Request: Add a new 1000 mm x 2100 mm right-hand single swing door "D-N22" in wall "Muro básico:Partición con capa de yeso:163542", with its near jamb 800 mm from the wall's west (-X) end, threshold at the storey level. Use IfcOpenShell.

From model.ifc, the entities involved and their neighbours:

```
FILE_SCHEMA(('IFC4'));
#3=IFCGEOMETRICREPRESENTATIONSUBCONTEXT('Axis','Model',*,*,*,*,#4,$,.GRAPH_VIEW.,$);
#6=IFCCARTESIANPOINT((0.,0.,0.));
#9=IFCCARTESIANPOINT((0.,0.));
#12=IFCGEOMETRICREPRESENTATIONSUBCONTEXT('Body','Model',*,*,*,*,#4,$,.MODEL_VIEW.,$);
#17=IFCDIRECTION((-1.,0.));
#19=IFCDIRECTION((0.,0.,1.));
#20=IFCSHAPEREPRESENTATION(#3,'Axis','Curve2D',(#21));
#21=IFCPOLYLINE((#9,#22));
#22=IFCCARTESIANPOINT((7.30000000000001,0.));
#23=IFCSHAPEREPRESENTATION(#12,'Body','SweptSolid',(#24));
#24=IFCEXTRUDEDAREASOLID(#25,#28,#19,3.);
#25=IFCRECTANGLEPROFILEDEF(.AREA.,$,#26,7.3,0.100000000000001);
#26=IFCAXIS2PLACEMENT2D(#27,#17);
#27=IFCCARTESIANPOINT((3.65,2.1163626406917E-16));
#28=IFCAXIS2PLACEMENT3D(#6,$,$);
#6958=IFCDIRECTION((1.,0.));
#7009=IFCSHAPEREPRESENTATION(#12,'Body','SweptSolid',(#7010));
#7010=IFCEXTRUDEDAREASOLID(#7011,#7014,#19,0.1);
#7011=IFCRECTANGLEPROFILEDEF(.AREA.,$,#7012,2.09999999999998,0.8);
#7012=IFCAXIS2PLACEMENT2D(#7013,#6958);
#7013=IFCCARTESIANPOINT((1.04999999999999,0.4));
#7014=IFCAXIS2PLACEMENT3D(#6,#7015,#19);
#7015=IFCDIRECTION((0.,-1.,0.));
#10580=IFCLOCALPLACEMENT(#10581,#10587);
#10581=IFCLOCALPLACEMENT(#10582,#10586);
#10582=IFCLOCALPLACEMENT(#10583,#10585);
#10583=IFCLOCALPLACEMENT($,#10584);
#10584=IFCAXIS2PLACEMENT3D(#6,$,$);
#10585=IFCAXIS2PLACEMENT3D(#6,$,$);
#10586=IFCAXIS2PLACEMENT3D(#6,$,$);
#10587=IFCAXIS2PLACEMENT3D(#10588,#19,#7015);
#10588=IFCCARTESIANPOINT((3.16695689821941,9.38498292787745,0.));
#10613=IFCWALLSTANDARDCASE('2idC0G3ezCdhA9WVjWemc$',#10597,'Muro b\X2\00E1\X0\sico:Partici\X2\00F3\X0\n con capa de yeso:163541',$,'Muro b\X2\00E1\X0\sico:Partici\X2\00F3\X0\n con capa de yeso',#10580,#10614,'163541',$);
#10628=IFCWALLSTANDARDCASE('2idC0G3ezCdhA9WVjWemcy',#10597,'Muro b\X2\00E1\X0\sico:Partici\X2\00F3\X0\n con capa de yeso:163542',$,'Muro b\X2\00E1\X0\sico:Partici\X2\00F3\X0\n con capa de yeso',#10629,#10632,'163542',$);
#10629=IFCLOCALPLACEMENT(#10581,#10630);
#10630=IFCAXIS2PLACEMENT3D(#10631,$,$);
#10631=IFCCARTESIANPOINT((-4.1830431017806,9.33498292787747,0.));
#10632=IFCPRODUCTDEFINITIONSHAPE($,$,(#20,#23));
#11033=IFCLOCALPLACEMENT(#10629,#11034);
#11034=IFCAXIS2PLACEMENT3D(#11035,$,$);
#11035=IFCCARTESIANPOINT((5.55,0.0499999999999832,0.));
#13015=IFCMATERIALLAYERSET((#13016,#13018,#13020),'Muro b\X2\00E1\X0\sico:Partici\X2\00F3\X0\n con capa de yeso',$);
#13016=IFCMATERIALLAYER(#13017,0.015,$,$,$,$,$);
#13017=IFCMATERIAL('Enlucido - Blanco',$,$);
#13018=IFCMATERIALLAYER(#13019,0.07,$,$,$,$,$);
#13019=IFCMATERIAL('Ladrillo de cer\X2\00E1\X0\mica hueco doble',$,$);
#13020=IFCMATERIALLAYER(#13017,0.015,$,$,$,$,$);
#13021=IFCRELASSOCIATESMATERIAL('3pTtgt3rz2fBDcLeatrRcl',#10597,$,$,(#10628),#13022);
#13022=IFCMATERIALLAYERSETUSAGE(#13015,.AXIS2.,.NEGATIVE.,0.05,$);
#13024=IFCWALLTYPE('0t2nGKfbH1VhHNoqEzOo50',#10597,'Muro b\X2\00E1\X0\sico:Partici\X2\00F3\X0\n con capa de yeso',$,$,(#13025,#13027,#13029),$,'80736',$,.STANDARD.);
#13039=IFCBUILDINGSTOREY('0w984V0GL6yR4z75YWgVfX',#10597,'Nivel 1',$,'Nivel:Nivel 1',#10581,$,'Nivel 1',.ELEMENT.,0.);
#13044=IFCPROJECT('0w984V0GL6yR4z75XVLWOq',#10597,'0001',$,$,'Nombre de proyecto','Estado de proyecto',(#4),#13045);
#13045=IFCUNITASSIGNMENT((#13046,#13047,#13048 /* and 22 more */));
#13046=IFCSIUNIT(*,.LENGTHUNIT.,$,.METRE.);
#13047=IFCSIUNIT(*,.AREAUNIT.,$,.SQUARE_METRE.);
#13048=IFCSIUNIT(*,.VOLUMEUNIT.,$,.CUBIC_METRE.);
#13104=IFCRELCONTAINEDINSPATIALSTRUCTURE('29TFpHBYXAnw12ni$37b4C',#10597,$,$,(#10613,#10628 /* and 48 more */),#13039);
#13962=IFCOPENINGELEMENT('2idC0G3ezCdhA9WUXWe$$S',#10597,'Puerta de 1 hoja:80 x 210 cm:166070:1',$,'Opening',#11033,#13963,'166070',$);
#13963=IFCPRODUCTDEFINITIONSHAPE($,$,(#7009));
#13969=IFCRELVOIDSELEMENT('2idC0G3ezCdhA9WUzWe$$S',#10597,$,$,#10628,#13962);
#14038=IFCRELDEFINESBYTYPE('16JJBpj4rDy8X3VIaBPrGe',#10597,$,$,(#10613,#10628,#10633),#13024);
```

```python
import numpy as np
import ifcopenshell
import ifcopenshell.api.feature
import ifcopenshell.api.geometry
import ifcopenshell.api.root
import ifcopenshell.api.spatial
import ifcopenshell.geom
import ifcopenshell.util.element
import ifcopenshell.util.placement
import ifcopenshell.util.representation
import ifcopenshell.util.shape
import ifcopenshell.util.unit

model = ifcopenshell.open("model.ifc")
unit_scale = ifcopenshell.util.unit.calculate_unit_scale(model)
settings = ifcopenshell.geom.settings()


def volume(element):
    """Net volume in cubic metres, openings subtracted."""
    shape = ifcopenshell.geom.create_shape(settings, element)
    return ifcopenshell.util.shape.get_volume(shape.geometry)


wall = model.by_guid("2idC0G3ezCdhA9WVjWemcy")
storey = ifcopenshell.util.element.get_container(wall, ifc_class="IfcBuildingStorey")
context = ifcopenshell.util.representation.get_context(model, "Model", "Body", "MODEL_VIEW")
before = volume(wall)

width, height, from_end, sill = 1, 2.1, 0.8, 0.0  # metres

# The wall runs along its own X axis, and the end named is its -X end.
wall_shape = ifcopenshell.geom.create_shape(settings, wall)
x, y, z = ifcopenshell.util.shape.get_vertices(wall_shape.geometry).T
start = x.min() + from_end
face, thickness = float(y.min()), float(y.max() - y.min())
wall_matrix = ifcopenshell.util.placement.get_local_placement(wall.ObjectPlacement)
level = ifcopenshell.util.placement.get_local_placement(storey.ObjectPlacement)[2, 3]


def in_wall(x, y):
    """Placement at x, y metres in the wall's axes, at sill height."""
    matrix = wall_matrix.copy()
    matrix[:, 3] = wall_matrix @ np.array([x / unit_scale, y / unit_scale, 0.0, 1.0])
    matrix[2, 3] = level + sill / unit_scale
    return matrix


# Opening: a box that overshoots both wall faces by 50 mm.
opening = ifcopenshell.api.root.create_entity(model, ifc_class="IfcOpeningElement", predefined_type="OPENING")
box = ifcopenshell.api.geometry.add_wall_representation(
    model, context=context, length=width, height=height, thickness=thickness + 0.1
)
ifcopenshell.api.geometry.assign_representation(model, product=opening, representation=box)
ifcopenshell.api.geometry.edit_object_placement(model, product=opening, matrix=in_wall(start, face - 0.05), is_si=False)
ifcopenshell.api.feature.add_feature(model, feature=opening, element=wall)

door = ifcopenshell.api.root.create_entity(model, ifc_class="IfcDoor", name="D-N22", predefined_type="DOOR")
door.OverallWidth, door.OverallHeight = width / unit_scale, height / unit_scale
door.OperationType = "SINGLE_SWING_RIGHT"
body = ifcopenshell.api.geometry.add_door_representation(
    model,
    context=context,
    overall_width=door.OverallWidth,
    overall_height=door.OverallHeight,
    operation_type="SINGLE_SWING_RIGHT",
    lining_properties={"LiningDepth": thickness / unit_scale, "ThresholdDepth": thickness / unit_scale},
)
ifcopenshell.api.geometry.assign_representation(model, product=door, representation=body)
ifcopenshell.api.spatial.assign_container(model, products=[door], relating_structure=storey)
ifcopenshell.api.feature.add_filling(model, opening=opening, element=door)

# The lining spans the wall, so the door starts at the wall face.
ifcopenshell.api.geometry.edit_object_placement(model, product=door, matrix=in_wall(start, face), is_si=False)

after = volume(wall)

print(f"wall volume {before:.3f} -> {after:.3f} m3")

model.write("model_v2.ifc")
```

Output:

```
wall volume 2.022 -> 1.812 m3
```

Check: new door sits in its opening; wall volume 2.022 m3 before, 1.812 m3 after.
